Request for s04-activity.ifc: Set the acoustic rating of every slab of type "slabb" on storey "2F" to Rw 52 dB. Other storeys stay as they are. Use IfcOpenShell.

First a look at what the model holds.

```python
import ifcopenshell
import ifcopenshell.util.element

model = ifcopenshell.open("s04-activity.ifc")
print(model.schema)
storey = next(s for s in model.by_type("IfcBuildingStorey") if s.Name == "2F")
slabs = [e for e in ifcopenshell.util.element.get_decomposition(storey) if e.is_a("IfcSlab")]
seen = {}
for e in slabs:
    element_type = ifcopenshell.util.element.get_type(e)
    key = (element_type.Name if element_type != e and element_type else None, ifcopenshell.util.element.get_pset(e, "Pset_SlabCommon", "AcousticRating"))
    seen[key] = seen.get(key, 0) + 1
for (name, value), count in sorted(seen.items(), key=str):
    print(count, "x", name, "|", value)
```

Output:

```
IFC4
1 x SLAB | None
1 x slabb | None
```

```python
import ifcopenshell
import ifcopenshell.api.pset
import ifcopenshell.util.element

model = ifcopenshell.open("s04-activity.ifc")

storey = next(s for s in model.by_type("IfcBuildingStorey") if s.Name == "2F")
slabs = [e for e in ifcopenshell.util.element.get_decomposition(storey) if e.is_a("IfcSlab")]

count = 0
for e in slabs:
    element_type = ifcopenshell.util.element.get_type(e)
    if element_type in (None, e) or element_type.Name != "slabb":
        continue
    # add_pset returns the element's existing set when there is one.
    pset = ifcopenshell.api.pset.add_pset(model, product=e, name="Pset_SlabCommon")
    ifcopenshell.api.pset.edit_pset(model, pset=pset, properties={"AcousticRating": "Rw 52 dB"})
    count += 1

print(count, "slabs updated")

model.write("s04-activity_rev.ifc")
```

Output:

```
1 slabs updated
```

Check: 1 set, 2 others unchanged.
